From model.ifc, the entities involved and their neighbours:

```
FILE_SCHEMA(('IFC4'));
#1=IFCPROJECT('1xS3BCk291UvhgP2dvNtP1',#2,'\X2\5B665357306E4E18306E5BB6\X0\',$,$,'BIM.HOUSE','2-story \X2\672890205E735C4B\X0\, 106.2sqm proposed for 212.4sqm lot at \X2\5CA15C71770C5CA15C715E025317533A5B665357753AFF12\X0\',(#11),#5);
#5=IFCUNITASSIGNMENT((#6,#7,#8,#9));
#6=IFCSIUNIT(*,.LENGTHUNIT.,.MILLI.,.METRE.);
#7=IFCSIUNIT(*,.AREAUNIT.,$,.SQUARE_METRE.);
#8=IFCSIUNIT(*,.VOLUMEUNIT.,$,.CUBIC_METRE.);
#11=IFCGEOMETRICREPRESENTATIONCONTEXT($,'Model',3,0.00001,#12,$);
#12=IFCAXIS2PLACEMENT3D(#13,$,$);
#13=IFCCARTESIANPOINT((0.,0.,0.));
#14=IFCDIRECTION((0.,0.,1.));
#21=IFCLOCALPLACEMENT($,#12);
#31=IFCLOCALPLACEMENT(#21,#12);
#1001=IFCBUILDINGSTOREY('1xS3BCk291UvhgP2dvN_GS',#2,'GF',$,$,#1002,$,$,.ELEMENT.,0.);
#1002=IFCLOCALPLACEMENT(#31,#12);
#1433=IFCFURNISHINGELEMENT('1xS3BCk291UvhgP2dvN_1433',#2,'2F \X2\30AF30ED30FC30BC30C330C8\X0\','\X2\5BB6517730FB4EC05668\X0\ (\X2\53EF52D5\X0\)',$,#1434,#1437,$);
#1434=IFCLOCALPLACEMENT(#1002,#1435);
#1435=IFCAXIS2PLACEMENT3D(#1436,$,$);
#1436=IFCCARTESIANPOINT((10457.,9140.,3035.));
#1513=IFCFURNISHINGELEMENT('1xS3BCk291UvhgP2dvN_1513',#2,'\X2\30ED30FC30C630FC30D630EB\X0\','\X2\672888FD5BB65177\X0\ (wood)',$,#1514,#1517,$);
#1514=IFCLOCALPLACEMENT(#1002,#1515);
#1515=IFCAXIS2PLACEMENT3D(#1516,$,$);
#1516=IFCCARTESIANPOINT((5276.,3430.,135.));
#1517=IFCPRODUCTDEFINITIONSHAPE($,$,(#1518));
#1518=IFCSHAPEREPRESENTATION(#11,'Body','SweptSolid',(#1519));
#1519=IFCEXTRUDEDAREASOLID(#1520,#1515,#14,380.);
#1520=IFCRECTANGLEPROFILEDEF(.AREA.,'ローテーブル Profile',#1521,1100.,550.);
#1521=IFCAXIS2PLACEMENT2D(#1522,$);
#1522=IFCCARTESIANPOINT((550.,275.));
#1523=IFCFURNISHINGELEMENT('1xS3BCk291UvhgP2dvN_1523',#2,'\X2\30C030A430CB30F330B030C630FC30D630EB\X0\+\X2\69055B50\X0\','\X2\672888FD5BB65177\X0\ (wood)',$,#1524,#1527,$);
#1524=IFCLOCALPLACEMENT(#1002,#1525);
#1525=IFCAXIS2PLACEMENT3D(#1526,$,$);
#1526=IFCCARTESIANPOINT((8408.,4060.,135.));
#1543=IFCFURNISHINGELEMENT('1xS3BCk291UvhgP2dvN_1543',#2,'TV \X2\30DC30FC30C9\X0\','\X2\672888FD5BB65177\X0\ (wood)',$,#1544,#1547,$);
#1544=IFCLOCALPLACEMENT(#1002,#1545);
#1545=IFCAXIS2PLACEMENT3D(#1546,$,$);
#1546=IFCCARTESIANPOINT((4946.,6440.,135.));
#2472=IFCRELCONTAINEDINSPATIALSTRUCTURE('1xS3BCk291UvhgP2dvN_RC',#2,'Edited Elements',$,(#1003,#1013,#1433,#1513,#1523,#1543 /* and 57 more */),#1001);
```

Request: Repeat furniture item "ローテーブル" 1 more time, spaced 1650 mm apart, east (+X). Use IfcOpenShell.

```python
import numpy as np
import ifcopenshell
import ifcopenshell.api.geometry
import ifcopenshell.api.root
import ifcopenshell.util.element
import ifcopenshell.util.placement
import ifcopenshell.util.unit

model = ifcopenshell.open("model.ifc")
unit_scale = ifcopenshell.util.unit.calculate_unit_scale(model)


def reuse_history(source, copy):
    """copy_class also copies each property set's owner history, people and application; keep the originals."""
    for rel in copy.IsDefinedBy:
        if rel.is_a("IfcRelDefinesByProperties") and (history := rel.RelatingPropertyDefinition.OwnerHistory):
            rel.RelatingPropertyDefinition.OwnerHistory = source.OwnerHistory
            ifcopenshell.util.element.remove_deep2(model, history)


source = model.by_guid("1xS3BCk291UvhgP2dvN_1513")
base = ifcopenshell.util.placement.get_local_placement(source.ObjectPlacement)
step = np.array([1.0, 0.0, 0.0]) * 1.65 / unit_scale

for i in range(1, 2):
    copy = ifcopenshell.api.root.copy_class(model, product=source)
    copy.Representation = ifcopenshell.util.element.copy_deep(
        model, source.Representation, exclude=["IfcGeometricRepresentationContext", "IfcRepresentationMap"]
    )
    reuse_history(source, copy)
    matrix = base.copy()
    matrix[:3, 3] += i * step
    print("added at", matrix[:3, 3].round(3) + 0.0)
    ifcopenshell.api.geometry.edit_object_placement(model, product=copy, matrix=matrix, is_si=False)

model.write("model_updated.ifc")
```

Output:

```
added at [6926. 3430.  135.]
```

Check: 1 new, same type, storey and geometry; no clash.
